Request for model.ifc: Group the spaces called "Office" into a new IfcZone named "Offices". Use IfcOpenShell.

First a look at what the model holds.

```python
import ifcopenshell

model = ifcopenshell.open("model.ifc")
print(model.schema)
seen = {}
for space in model.by_type("IfcSpace"):
    seen[space.LongName] = seen.get(space.LongName, 0) + 1
for name, count in sorted(seen.items(), key=str):
    print(count, "x", name)
print("zones:", [z.Name for z in model.by_type("IfcZone")][:20])
```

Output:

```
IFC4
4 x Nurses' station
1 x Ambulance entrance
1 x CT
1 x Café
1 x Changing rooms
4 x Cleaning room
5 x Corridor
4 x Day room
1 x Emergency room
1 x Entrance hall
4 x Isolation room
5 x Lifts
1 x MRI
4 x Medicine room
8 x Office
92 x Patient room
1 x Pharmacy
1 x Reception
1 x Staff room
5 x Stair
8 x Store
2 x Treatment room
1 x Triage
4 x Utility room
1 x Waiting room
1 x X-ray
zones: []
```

```python
import ifcopenshell
import ifcopenshell.api.group
import ifcopenshell.api.root

model = ifcopenshell.open("model.ifc")

names = {"Office"}
spaces = [s for s in model.by_type("IfcSpace") if s.LongName in names]

zone = ifcopenshell.api.root.create_entity(model, ifc_class="IfcZone", name="Offices")
ifcopenshell.api.group.assign_group(model, products=spaces, group=zone)
print(len(spaces), "spaces in", zone.Name)

model.write("model_v2.ifc")
```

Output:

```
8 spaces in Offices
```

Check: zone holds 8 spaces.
